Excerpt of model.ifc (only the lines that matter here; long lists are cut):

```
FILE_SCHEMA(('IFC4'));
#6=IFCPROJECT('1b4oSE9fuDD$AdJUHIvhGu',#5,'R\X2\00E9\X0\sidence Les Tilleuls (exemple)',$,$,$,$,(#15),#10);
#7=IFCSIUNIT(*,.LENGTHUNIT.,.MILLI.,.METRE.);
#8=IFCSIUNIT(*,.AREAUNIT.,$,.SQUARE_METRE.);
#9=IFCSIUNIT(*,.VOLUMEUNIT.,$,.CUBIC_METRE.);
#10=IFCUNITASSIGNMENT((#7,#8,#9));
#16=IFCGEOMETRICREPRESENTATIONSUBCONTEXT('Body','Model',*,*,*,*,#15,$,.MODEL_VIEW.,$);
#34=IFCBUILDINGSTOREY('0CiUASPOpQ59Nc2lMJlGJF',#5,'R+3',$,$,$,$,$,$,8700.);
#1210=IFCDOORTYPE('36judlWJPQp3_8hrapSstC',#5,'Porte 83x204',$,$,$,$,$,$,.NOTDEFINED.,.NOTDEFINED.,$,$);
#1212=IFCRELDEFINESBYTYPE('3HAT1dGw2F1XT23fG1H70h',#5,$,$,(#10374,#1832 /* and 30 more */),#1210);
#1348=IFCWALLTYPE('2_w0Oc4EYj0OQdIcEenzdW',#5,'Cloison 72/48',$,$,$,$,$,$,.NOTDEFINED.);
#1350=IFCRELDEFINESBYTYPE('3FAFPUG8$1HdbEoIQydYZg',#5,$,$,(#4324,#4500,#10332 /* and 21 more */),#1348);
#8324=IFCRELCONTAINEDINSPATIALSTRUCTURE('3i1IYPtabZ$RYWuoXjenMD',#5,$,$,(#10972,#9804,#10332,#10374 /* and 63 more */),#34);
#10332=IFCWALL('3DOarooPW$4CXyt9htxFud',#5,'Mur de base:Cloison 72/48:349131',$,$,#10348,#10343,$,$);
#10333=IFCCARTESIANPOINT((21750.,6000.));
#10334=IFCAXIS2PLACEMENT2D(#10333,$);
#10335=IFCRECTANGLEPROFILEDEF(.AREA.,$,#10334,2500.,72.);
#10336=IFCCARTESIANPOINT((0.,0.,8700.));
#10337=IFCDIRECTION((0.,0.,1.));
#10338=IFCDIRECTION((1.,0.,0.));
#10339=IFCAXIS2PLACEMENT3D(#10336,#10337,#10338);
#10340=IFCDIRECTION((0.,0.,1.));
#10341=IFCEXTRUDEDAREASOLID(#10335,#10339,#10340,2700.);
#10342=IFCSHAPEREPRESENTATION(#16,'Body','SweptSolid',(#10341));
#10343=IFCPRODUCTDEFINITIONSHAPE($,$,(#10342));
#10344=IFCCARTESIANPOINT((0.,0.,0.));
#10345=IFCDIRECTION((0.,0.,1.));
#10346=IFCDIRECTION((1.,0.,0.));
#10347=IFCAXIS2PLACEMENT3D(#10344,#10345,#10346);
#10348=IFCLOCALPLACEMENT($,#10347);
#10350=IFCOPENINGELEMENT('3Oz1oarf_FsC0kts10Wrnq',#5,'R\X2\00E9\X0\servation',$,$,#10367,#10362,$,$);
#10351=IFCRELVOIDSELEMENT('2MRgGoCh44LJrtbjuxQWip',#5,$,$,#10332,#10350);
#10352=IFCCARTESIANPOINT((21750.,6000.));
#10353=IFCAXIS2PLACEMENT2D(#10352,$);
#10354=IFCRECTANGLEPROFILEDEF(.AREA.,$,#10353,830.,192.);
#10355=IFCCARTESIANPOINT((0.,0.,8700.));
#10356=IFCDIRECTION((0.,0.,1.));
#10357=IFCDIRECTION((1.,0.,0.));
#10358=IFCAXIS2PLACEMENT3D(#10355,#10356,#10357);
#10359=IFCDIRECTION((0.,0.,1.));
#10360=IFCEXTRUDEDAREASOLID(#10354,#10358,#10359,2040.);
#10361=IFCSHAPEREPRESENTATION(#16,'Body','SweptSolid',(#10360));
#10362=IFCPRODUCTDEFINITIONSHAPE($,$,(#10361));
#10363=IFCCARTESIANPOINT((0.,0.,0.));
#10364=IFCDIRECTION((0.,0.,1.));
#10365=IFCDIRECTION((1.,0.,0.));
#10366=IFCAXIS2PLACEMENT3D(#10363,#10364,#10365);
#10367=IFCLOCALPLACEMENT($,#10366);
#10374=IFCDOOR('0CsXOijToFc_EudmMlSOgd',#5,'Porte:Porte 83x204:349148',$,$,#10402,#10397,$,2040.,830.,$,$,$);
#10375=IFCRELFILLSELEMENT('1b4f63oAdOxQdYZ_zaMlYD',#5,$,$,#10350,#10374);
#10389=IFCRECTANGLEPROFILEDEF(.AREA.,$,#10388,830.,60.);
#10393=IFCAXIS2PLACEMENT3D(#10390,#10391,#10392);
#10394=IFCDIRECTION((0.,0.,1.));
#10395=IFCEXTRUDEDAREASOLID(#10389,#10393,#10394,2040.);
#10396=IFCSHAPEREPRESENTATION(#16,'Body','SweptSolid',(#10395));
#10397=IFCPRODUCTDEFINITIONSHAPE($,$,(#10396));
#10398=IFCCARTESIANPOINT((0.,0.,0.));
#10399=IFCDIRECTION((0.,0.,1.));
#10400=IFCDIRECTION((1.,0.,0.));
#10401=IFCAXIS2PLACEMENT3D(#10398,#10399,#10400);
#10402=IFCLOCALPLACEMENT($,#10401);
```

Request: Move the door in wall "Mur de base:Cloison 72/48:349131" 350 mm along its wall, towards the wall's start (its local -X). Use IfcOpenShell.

```python
import ifcopenshell
import ifcopenshell.api.geometry
import ifcopenshell.util.placement
import ifcopenshell.util.unit

model = ifcopenshell.open("model.ifc")
unit_scale = ifcopenshell.util.unit.calculate_unit_scale(model)

door = model.by_guid("0CsXOijToFc_EudmMlSOgd")
opening = door.FillsVoids[0].RelatingOpeningElement
wall = opening.VoidsElements[0].RelatingBuildingElement

wall_matrix = ifcopenshell.util.placement.get_local_placement(wall.ObjectPlacement)
shift = wall_matrix[:3, 0] * -0.35 / unit_scale
before = ifcopenshell.util.placement.get_local_placement(door.ObjectPlacement)[:3, 3].copy()

# The door is not placed relative to its opening, so move both.
for product in (opening, door):
    matrix = ifcopenshell.util.placement.get_local_placement(product.ObjectPlacement)
    matrix[:3, 3] += shift
    ifcopenshell.api.geometry.edit_object_placement(model, product=product, matrix=matrix, is_si=False)

after = ifcopenshell.util.placement.get_local_placement(door.ObjectPlacement)[:3, 3]
print("door moved by", (after - before).round(3) + 0.0)

model.write("model_rev.ifc")
```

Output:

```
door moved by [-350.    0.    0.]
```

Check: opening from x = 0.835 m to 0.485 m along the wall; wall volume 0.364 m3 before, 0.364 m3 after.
